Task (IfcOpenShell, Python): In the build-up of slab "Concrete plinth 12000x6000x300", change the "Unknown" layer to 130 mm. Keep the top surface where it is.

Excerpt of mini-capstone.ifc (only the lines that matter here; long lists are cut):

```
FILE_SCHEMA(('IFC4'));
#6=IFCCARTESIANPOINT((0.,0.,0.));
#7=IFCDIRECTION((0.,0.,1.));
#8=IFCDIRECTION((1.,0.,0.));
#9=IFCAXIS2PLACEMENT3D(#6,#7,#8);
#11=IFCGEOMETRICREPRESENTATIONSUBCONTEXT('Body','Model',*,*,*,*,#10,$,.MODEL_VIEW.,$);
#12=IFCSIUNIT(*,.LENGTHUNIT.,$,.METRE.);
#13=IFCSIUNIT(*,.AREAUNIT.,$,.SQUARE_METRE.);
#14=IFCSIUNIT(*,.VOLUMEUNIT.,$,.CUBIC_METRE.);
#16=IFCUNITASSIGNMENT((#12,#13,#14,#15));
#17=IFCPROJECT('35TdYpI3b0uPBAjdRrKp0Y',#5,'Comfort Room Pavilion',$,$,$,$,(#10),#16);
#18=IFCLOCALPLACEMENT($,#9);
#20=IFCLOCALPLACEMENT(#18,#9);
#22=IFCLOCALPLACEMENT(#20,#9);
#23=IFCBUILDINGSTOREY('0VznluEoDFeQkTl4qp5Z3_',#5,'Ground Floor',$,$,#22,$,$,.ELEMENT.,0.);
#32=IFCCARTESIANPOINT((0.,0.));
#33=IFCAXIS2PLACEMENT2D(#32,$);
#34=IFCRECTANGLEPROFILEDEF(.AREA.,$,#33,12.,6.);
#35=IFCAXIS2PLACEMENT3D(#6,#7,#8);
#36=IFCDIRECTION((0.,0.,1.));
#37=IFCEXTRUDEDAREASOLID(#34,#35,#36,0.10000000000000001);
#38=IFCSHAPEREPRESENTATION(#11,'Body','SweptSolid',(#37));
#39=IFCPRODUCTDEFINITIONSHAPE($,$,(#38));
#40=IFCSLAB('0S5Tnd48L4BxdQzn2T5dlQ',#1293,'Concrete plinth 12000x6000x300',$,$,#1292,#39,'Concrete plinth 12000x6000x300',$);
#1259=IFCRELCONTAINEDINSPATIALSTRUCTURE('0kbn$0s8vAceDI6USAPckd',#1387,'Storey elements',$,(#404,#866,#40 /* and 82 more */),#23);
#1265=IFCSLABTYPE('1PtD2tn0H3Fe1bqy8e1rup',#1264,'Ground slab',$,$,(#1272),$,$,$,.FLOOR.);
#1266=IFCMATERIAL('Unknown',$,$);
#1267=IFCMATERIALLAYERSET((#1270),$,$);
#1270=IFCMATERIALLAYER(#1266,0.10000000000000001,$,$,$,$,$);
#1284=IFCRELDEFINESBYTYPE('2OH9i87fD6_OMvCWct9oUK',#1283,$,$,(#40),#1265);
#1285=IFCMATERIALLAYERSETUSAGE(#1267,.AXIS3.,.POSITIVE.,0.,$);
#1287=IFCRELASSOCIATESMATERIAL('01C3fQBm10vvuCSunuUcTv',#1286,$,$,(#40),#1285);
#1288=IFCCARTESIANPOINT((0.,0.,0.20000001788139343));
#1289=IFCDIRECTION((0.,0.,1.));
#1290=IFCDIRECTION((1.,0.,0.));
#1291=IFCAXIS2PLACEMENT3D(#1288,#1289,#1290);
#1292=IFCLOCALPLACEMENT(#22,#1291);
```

```python
import ifcopenshell
import ifcopenshell.util.element
import ifcopenshell.util.representation
import ifcopenshell.util.unit

model = ifcopenshell.open("mini-capstone.ifc")
unit_scale = ifcopenshell.util.unit.calculate_unit_scale(model)

layer_set = model.by_id(1267)
layer = next(l for l in layer_set.MaterialLayers if l.Material and l.Material.Name == "Unknown")
change = 0.13 / unit_scale - layer.LayerThickness
layer.LayerThickness += change

# Geometry does not follow the layer set by itself.
slabs = [e for e in ifcopenshell.util.element.get_elements_by_material(model, layer_set) if e.is_a("IfcSlab")]
for slab in sorted(slabs, key=lambda e: e.id()):
    body = ifcopenshell.util.representation.get_representation(slab, "Model", "Body")
    solid = body.Items[0]
    old_depth = solid.Depth
    solid.Depth += change
    # Extruded upwards: lower the start of the extrusion so the top stays.
    x, y, z = solid.Position.Location.Coordinates
    solid.Position.Location = model.createIfcCartesianPoint((x, y, z - change))
    print(slab.id(), f"{old_depth:g} -> {solid.Depth:g}")

# The layers are counted up from the underside, which has moved.
for usage in {ifcopenshell.util.element.get_material(slab) for slab in slabs}:
    usage.OffsetFromReferenceLine -= change

model.write("mini-capstone_updated.ifc")
```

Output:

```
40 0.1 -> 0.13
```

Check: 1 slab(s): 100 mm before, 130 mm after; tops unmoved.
